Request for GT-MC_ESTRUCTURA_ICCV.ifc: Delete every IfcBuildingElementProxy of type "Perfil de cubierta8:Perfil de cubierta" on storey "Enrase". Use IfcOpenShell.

First a look at what the model holds.

```python
import ifcopenshell
import ifcopenshell.util.element

model = ifcopenshell.open("GT-MC_ESTRUCTURA_ICCV.ifc")
print(model.schema)
storey = next(s for s in model.by_type("IfcBuildingStorey") if s.Name == "Enrase")
proxies = [e for e in ifcopenshell.util.element.get_decomposition(storey) if e.is_a("IfcBuildingElementProxy")]
seen = {}
for e in proxies:
    element_type = ifcopenshell.util.element.get_type(e)
    name = element_type.Name if element_type not in (None, e) else None
    seen[name] = seen.get(name, 0) + 1
for name, count in sorted(seen.items(), key=str):
    print(count, "x", name)
```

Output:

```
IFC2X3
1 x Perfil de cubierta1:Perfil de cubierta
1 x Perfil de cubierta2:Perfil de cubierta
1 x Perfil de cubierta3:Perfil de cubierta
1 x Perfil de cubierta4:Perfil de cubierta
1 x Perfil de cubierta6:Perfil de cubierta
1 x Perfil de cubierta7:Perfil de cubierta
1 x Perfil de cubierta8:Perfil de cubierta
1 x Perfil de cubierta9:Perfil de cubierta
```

```python
import ifcopenshell
import ifcopenshell.api.root
import ifcopenshell.util.element

model = ifcopenshell.open("GT-MC_ESTRUCTURA_ICCV.ifc")

storey = next(s for s in model.by_type("IfcBuildingStorey") if s.Name == "Enrase")
proxies = [e for e in ifcopenshell.util.element.get_decomposition(storey) if e.is_a("IfcBuildingElementProxy")]
targets = [e for e in proxies if (t := ifcopenshell.util.element.get_type(e)) not in (None, e) and t.Name == "Perfil de cubierta8:Perfil de cubierta"]

for e in targets:
    ifcopenshell.api.root.remove_product(model, product=e)
print(len(targets), "removed")

model.write("GT-MC_ESTRUCTURA_ICCV_edited.ifc")
```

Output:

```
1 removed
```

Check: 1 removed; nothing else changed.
